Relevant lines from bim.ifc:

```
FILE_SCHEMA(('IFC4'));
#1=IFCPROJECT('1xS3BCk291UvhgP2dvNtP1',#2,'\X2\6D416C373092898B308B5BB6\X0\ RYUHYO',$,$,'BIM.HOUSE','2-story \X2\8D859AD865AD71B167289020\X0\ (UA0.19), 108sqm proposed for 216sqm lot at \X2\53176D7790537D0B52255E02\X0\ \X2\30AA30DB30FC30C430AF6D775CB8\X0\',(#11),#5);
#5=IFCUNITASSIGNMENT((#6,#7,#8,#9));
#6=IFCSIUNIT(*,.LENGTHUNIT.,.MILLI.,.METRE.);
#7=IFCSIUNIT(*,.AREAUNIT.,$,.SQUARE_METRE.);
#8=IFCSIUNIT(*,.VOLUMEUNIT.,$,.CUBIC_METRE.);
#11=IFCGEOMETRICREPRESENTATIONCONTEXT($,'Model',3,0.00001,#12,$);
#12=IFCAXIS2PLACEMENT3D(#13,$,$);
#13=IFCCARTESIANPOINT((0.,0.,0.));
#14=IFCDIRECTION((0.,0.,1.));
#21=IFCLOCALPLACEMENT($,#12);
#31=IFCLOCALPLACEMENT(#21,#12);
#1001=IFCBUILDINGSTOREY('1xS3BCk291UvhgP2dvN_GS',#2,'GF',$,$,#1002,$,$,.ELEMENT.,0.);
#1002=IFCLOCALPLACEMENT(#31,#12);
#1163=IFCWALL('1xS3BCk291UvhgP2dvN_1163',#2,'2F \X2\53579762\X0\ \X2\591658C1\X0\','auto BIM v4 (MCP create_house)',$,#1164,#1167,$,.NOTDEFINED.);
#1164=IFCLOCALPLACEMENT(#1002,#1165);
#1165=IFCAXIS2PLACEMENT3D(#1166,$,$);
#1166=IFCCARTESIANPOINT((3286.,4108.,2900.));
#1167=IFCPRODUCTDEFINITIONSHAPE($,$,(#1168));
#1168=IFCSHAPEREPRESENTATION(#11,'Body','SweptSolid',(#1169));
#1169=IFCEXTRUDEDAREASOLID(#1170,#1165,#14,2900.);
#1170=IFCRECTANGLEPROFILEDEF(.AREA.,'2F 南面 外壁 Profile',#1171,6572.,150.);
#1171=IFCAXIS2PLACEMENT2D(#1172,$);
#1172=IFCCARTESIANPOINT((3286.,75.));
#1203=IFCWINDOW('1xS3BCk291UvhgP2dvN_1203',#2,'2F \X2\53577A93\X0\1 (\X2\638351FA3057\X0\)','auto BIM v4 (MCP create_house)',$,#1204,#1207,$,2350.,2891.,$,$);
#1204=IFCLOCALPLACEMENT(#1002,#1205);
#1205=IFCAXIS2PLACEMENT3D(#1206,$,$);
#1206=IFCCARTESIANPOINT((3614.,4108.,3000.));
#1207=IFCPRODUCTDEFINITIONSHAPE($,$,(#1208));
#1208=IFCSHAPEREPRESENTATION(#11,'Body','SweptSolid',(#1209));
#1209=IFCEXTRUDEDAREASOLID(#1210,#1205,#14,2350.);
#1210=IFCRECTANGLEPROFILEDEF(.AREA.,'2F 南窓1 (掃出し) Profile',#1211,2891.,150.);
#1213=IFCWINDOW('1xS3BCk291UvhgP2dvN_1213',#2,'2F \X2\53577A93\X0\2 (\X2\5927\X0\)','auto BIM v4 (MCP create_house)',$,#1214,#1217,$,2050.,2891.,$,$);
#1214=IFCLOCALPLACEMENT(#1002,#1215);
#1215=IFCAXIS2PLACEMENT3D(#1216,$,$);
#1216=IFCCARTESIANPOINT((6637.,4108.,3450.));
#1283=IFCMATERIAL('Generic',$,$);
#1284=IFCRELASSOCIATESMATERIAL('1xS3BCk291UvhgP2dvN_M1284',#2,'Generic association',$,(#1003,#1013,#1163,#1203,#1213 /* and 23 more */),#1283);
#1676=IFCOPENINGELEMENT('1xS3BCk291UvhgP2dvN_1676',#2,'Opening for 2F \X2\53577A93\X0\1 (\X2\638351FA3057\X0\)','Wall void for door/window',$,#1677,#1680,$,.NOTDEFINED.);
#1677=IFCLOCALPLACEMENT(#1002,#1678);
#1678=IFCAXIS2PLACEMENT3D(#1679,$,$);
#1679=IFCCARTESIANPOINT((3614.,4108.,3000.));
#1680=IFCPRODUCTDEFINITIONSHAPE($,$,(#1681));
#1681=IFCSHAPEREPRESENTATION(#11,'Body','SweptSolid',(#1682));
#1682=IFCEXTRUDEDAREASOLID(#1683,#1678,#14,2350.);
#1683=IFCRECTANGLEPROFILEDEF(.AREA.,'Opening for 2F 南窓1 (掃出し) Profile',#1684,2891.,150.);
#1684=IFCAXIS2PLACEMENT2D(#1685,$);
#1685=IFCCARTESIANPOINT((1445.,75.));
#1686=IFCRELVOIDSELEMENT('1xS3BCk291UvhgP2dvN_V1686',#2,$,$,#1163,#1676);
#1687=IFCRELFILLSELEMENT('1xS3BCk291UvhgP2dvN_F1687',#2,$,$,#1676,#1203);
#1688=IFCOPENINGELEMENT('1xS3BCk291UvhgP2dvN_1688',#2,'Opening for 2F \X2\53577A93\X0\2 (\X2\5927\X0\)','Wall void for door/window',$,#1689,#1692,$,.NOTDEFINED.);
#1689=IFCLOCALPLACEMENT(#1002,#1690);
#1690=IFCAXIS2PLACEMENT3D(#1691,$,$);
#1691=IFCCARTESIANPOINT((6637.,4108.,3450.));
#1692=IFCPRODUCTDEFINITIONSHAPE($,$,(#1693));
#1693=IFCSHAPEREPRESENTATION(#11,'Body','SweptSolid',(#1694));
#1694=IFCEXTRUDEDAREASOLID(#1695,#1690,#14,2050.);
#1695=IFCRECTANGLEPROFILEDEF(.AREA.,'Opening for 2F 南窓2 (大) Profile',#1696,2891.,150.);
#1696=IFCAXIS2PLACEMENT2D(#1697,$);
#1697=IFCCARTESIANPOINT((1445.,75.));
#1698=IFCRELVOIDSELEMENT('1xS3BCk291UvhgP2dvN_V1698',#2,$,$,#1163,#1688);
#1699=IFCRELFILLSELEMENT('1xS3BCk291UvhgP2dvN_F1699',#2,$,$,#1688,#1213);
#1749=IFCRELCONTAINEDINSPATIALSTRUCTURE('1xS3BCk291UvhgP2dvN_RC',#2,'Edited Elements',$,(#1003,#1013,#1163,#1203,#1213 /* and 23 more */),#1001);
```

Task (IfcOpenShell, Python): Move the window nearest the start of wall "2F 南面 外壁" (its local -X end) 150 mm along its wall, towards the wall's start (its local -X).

```python
import ifcopenshell
import ifcopenshell.api.geometry
import ifcopenshell.util.placement
import ifcopenshell.util.unit

model = ifcopenshell.open("bim.ifc")
unit_scale = ifcopenshell.util.unit.calculate_unit_scale(model)

window = model.by_guid("1xS3BCk291UvhgP2dvN_1203")
opening = window.FillsVoids[0].RelatingOpeningElement
wall = opening.VoidsElements[0].RelatingBuildingElement

wall_matrix = ifcopenshell.util.placement.get_local_placement(wall.ObjectPlacement)
shift = wall_matrix[:3, 0] * -0.15 / unit_scale
before = ifcopenshell.util.placement.get_local_placement(window.ObjectPlacement)[:3, 3].copy()

# The window is not placed relative to its opening, so move both.
for product in (opening, window):
    matrix = ifcopenshell.util.placement.get_local_placement(product.ObjectPlacement)
    matrix[:3, 3] += shift
    ifcopenshell.api.geometry.edit_object_placement(model, product=product, matrix=matrix, is_si=False)

after = ifcopenshell.util.placement.get_local_placement(window.ObjectPlacement)[:3, 3]
print("window moved by", (after - before).round(3) + 0.0)

model.write("bim_rev.ifc")
```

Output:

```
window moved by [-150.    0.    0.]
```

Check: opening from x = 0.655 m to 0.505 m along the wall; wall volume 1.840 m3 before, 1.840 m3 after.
